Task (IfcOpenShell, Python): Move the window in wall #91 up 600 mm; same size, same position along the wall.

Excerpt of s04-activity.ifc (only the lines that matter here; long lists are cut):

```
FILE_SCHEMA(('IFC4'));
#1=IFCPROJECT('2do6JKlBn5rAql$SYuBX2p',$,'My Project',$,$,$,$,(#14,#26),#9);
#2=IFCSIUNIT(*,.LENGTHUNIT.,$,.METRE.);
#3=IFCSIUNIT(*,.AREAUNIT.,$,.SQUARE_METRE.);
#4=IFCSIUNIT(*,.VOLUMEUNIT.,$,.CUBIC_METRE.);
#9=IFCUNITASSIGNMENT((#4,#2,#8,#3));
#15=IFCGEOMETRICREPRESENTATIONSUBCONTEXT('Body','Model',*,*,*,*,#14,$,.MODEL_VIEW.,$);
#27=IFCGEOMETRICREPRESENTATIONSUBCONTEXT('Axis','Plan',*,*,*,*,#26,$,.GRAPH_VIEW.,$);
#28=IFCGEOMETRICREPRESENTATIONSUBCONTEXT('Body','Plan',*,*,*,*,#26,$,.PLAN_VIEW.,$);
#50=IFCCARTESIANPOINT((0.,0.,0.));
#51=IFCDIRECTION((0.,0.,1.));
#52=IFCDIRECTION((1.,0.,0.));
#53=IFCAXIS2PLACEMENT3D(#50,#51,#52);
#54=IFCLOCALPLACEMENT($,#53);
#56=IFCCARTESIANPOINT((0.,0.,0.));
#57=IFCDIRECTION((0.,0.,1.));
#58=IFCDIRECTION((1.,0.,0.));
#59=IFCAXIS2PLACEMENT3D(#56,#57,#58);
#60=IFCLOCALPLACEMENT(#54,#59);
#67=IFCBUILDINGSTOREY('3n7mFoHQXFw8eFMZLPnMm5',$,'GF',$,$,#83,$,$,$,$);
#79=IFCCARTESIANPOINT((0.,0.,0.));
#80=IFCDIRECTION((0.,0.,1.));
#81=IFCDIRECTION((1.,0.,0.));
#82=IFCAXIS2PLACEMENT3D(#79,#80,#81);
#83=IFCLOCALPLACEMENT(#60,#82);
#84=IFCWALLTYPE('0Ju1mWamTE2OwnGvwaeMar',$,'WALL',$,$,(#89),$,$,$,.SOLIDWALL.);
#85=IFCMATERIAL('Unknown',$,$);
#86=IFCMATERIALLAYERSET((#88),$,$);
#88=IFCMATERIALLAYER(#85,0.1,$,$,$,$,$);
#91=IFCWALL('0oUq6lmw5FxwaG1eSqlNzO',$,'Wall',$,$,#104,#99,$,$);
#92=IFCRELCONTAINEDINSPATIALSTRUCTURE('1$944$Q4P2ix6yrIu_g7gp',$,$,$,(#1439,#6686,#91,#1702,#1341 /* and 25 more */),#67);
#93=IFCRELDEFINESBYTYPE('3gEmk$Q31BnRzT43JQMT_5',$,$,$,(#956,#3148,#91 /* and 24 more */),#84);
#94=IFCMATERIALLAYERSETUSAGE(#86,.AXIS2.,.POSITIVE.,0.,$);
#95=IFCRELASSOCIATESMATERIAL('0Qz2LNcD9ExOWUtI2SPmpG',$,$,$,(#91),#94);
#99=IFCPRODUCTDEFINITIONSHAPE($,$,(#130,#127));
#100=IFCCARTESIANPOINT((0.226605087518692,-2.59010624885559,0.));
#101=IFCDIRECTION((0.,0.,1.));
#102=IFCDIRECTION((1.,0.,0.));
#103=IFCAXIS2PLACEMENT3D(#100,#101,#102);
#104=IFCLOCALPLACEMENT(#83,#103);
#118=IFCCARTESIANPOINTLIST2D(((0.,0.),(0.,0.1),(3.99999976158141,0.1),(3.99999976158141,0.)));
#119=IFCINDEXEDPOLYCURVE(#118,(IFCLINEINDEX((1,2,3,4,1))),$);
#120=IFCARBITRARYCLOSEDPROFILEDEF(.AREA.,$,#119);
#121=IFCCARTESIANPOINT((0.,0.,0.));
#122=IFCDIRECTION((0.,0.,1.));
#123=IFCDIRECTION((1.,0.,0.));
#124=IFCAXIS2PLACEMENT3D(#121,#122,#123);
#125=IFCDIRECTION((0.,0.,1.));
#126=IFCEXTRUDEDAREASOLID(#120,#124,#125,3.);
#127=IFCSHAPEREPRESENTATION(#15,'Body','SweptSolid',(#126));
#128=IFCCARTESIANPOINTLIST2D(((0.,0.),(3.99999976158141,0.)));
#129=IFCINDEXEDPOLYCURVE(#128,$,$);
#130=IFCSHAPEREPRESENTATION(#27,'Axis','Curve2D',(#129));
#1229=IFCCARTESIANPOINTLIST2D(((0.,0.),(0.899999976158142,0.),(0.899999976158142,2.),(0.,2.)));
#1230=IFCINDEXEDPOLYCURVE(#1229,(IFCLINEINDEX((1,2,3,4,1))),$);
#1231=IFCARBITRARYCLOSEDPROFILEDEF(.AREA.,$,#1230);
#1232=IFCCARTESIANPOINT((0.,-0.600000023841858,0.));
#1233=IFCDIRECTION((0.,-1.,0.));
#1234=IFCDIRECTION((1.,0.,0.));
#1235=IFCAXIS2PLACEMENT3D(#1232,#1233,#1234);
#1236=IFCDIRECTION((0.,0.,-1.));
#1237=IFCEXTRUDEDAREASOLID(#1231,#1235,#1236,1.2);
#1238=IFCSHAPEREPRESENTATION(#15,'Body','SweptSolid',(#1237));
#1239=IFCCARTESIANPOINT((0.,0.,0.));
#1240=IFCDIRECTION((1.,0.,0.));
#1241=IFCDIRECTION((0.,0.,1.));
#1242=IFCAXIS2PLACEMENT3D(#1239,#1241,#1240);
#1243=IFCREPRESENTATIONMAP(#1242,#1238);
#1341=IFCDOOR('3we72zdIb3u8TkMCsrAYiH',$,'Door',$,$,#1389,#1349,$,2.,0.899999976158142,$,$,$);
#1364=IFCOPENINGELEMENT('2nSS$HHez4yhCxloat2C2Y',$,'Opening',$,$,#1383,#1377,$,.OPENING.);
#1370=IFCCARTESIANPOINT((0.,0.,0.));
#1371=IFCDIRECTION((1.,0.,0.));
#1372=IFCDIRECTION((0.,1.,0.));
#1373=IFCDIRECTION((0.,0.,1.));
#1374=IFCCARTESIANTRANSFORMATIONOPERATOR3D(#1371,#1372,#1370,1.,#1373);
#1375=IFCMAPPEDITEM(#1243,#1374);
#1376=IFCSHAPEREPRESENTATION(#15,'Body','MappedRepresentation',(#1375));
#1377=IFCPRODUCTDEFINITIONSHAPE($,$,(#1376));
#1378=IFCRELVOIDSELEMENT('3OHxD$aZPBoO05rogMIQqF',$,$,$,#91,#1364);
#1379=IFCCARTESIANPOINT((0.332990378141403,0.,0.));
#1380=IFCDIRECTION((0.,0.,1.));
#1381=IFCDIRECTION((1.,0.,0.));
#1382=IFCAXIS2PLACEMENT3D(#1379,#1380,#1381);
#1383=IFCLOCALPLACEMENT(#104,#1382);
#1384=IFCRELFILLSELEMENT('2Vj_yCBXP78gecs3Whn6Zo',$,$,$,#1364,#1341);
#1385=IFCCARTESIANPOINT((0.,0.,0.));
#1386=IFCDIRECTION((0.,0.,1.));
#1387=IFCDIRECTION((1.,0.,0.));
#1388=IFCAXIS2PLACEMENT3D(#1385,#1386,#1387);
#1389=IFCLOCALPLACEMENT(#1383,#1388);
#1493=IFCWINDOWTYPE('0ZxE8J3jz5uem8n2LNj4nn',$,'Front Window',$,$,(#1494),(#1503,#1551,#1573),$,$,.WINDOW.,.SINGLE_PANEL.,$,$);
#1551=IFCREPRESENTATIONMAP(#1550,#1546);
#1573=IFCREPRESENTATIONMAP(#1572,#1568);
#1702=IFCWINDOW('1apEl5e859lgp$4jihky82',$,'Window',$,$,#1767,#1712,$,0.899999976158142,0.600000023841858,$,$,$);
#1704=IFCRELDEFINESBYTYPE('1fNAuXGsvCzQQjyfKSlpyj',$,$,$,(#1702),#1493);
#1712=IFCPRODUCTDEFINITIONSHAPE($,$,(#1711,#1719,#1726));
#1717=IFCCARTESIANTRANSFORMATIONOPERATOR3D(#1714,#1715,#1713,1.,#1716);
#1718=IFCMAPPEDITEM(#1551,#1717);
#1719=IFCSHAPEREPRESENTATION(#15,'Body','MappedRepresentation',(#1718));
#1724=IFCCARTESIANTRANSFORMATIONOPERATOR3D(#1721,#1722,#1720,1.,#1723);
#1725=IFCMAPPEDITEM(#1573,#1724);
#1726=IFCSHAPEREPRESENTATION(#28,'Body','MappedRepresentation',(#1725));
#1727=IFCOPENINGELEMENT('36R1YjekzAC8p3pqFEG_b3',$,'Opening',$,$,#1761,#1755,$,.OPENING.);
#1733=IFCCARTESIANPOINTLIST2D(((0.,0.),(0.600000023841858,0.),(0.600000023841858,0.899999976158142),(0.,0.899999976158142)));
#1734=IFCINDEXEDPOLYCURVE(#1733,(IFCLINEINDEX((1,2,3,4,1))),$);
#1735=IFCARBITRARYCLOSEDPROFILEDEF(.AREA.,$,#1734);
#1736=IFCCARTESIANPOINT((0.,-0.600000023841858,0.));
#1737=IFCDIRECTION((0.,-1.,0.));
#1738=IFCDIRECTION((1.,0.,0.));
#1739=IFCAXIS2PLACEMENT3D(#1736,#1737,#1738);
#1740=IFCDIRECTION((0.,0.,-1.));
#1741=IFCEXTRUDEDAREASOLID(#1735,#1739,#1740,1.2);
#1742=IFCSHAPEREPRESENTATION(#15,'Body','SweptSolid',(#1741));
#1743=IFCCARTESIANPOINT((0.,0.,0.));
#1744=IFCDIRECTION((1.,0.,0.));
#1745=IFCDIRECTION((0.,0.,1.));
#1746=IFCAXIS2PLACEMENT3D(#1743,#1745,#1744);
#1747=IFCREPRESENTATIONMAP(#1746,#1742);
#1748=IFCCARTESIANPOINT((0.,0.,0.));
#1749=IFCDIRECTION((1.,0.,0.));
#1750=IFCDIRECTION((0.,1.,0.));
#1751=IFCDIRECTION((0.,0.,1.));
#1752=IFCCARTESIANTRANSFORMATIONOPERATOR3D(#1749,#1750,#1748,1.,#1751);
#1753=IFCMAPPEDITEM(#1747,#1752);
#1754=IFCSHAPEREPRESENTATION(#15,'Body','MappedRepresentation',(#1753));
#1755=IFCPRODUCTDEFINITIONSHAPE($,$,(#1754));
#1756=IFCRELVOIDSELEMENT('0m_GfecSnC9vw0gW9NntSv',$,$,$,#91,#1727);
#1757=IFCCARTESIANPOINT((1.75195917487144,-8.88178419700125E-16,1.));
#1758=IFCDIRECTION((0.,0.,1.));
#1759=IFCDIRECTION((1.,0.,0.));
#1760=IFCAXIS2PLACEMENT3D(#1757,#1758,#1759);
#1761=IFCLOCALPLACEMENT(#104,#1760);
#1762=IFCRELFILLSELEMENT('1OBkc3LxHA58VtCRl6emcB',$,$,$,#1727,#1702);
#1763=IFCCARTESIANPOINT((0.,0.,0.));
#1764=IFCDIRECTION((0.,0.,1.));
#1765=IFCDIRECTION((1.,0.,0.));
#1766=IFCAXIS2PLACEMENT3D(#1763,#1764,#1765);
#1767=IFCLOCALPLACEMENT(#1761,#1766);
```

```python
import numpy as np
import ifcopenshell
import ifcopenshell.api.geometry
import ifcopenshell.util.placement
import ifcopenshell.util.unit

model = ifcopenshell.open("s04-activity.ifc")
unit_scale = ifcopenshell.util.unit.calculate_unit_scale(model)

window = model.by_guid("1apEl5e859lgp$4jihky82")
opening = window.FillsVoids[0].RelatingOpeningElement
dz = 0.6

shift = np.array([0.0, 0.0, dz])
# The window is placed relative to its opening, so it follows when the opening moves.
matrix = ifcopenshell.util.placement.get_local_placement(opening.ObjectPlacement)
matrix[:3, 3] += shift
ifcopenshell.api.geometry.edit_object_placement(
    model, product=opening, matrix=matrix, is_si=False, should_transform_children=True
)

print(f"moved by {dz * unit_scale:+.3f} m")

model.write("s04-activity_v2.ifc")
```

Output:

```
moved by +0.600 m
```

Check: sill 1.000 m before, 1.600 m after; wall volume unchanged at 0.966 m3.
